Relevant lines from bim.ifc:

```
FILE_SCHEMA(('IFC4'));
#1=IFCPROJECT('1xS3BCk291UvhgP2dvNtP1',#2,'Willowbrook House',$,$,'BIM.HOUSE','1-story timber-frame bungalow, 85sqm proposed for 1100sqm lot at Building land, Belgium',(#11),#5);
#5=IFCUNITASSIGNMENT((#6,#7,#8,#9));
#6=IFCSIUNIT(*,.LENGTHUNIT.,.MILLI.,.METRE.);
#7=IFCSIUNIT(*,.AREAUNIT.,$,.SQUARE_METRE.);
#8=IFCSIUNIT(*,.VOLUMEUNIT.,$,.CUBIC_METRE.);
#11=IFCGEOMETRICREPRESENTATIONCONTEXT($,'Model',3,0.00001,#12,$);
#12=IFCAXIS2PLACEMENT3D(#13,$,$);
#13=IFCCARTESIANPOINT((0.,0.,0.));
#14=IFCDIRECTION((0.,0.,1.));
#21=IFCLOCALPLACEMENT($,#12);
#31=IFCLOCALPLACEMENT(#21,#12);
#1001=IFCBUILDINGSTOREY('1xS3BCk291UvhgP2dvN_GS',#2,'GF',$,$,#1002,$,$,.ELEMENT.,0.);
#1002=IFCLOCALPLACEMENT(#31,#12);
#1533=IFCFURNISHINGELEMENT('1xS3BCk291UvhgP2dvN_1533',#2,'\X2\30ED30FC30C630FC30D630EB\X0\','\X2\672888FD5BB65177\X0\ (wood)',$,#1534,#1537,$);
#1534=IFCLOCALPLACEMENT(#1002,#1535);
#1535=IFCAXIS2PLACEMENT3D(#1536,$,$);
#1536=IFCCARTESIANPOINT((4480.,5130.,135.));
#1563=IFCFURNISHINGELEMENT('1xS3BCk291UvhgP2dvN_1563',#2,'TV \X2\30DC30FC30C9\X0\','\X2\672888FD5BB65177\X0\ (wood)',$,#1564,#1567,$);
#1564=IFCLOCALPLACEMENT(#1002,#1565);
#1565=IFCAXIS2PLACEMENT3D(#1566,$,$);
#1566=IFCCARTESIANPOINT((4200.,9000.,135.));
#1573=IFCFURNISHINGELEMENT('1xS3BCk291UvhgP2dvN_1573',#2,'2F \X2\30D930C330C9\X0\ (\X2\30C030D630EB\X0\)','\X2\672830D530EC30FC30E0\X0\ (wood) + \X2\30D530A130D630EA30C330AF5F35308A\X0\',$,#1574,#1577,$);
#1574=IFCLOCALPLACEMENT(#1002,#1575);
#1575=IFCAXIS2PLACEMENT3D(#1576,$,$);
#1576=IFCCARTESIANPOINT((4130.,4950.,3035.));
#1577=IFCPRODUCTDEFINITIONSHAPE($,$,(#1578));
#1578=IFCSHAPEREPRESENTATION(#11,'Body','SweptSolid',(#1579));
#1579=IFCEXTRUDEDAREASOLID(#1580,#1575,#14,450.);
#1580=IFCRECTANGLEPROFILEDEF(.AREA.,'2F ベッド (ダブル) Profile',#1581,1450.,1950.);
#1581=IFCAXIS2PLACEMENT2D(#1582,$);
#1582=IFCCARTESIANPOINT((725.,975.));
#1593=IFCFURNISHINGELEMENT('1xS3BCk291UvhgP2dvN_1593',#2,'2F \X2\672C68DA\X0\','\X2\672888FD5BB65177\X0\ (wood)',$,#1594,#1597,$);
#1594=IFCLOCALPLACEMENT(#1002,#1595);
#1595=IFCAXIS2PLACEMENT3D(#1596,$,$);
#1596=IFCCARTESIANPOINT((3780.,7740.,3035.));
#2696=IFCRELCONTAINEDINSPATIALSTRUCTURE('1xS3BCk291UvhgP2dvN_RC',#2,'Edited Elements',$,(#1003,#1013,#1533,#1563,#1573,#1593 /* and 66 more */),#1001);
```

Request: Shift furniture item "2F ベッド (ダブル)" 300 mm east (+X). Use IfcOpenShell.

```python
import ifcopenshell
import ifcopenshell.api.geometry
import ifcopenshell.util.placement
import ifcopenshell.util.unit

model = ifcopenshell.open("bim.ifc")
unit_scale = ifcopenshell.util.unit.calculate_unit_scale(model)

item = model.by_guid("1xS3BCk291UvhgP2dvN_1573")
matrix = ifcopenshell.util.placement.get_local_placement(item.ObjectPlacement)
matrix[0, 3] += 0.3 / unit_scale
ifcopenshell.api.geometry.edit_object_placement(model, product=item, matrix=matrix, is_si=False)

print(ifcopenshell.util.placement.get_local_placement(item.ObjectPlacement).round(3) + 0.0)

model.write("bim-out.ifc")
```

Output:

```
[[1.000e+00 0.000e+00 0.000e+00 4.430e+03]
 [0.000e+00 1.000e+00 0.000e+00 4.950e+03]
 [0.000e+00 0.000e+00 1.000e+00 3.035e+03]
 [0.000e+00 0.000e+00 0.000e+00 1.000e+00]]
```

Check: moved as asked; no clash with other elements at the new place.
